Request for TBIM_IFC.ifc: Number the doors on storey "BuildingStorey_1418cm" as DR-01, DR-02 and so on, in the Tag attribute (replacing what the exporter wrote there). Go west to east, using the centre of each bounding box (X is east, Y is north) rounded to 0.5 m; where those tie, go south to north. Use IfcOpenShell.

First a look at what the model holds.

```python
import ifcopenshell
import ifcopenshell.util.element
import ifcopenshell.util.placement

model = ifcopenshell.open("TBIM_IFC.ifc")
print(model.schema)
storey = next(s for s in model.by_type("IfcBuildingStorey") if s.Name == "BuildingStorey_1418cm")
doors = [e for e in ifcopenshell.util.element.get_decomposition(storey) if e.is_a("IfcDoor")]
for e in sorted(doors, key=lambda e: e.id()):
    origin = ifcopenshell.util.placement.get_local_placement(e.ObjectPlacement)[:3, 3]
    print(e.id(), e.Tag, e.Name, origin.round(2) + 0.0, sep=" | ")
```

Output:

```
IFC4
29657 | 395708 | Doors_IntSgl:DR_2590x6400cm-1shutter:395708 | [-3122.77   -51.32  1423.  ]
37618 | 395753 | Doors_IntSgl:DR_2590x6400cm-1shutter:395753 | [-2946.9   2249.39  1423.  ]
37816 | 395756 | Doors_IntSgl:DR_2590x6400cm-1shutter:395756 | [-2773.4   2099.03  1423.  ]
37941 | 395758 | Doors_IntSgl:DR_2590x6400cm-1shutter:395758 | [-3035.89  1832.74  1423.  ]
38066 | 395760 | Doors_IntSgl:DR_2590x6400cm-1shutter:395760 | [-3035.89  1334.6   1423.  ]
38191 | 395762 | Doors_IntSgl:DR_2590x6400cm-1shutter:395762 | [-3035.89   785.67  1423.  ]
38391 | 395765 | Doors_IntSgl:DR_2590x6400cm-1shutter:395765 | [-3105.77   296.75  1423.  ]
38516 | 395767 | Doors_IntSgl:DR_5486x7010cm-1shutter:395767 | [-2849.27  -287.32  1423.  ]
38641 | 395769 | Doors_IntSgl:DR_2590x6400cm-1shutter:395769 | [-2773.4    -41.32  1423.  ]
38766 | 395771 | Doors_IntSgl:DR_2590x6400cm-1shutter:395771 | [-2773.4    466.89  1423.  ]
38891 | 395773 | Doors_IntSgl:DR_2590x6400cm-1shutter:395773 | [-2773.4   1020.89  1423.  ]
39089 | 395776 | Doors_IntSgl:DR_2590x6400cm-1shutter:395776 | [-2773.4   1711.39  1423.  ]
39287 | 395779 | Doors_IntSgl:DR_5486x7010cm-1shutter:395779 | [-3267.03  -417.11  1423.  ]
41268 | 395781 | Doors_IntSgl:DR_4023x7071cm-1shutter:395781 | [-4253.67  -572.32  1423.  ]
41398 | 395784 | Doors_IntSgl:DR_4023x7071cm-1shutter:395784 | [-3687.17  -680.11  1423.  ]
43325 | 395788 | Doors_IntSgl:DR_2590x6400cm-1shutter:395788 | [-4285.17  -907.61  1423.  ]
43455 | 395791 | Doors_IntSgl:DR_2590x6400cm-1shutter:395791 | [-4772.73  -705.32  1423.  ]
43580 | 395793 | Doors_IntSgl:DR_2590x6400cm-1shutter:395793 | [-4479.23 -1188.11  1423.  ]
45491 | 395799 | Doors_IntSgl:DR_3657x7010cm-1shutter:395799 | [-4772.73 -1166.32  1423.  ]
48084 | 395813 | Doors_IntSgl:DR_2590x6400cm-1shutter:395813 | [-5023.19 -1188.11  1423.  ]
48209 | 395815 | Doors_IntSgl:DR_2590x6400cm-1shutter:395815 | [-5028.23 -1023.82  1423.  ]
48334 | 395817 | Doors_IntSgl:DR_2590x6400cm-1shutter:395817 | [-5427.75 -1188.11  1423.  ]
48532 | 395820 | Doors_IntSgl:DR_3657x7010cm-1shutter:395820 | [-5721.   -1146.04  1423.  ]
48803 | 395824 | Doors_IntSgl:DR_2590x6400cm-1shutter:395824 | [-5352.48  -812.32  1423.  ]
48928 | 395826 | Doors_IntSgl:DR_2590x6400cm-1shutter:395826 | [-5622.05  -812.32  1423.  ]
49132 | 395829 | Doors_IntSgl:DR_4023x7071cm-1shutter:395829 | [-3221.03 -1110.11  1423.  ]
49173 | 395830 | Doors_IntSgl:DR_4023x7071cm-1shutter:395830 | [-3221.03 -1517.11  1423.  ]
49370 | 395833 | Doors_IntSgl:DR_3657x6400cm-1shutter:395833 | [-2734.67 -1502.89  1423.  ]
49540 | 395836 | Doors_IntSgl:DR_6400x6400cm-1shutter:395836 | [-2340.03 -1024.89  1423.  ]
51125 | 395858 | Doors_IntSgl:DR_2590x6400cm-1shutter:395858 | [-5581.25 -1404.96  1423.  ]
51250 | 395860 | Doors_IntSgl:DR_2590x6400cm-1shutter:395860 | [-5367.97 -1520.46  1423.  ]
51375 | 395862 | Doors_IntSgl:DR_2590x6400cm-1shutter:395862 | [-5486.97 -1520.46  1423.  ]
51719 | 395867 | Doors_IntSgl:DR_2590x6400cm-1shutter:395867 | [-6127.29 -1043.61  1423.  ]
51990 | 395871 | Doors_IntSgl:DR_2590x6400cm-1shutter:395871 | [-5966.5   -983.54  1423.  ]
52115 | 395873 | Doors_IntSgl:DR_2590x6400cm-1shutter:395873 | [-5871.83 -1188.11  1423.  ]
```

```python
import ifcopenshell
import ifcopenshell.geom
import ifcopenshell.util.element
import ifcopenshell.util.shape

model = ifcopenshell.open("TBIM_IFC.ifc")
settings = ifcopenshell.geom.settings()
settings.set("use-world-coords", True)


def centre(element):
    shape = ifcopenshell.geom.create_shape(settings, element)
    return ifcopenshell.util.shape.get_bbox_centroid(shape.geometry)


storey = next(s for s in model.by_type("IfcBuildingStorey") if s.Name == "BuildingStorey_1418cm")
doors = [e for e in ifcopenshell.util.element.get_decomposition(storey) if e.is_a("IfcDoor")]

# Insertion points can sit at a corner or the storey origin, so sort by the geometry (in metres).
centres = {e: centre(e) for e in doors}
doors.sort(key=lambda e: (round(centres[e][0] / 0.5), centres[e][1]))

for i, e in enumerate(doors, start=1):
    number = f"DR-{i:02d}"
    e.Tag = number
    print(e.id(), number)

model.write("TBIM_IFC_rev.ifc")
```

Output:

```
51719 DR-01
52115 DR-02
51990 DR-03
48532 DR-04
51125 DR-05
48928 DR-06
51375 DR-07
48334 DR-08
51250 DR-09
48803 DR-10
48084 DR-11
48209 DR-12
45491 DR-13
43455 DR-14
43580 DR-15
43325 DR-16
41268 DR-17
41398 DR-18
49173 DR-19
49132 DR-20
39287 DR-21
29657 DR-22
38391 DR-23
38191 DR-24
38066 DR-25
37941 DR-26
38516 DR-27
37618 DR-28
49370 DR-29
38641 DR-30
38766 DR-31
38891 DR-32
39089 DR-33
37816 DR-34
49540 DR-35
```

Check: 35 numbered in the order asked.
